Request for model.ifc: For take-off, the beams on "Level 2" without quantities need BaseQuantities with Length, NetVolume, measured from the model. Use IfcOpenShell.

First a look at what the model holds.

```python
import ifcopenshell
import ifcopenshell.util.element
import ifcopenshell.util.unit

model = ifcopenshell.open("model.ifc")
print(model.schema)
for unit_type in ("LENGTHUNIT", "AREAUNIT", "VOLUMEUNIT"):
    print(unit_type, ifcopenshell.util.unit.calculate_unit_scale(model, unit_type))
storey = next(s for s in model.by_type("IfcBuildingStorey") if s.Name == "Level 2")
beams = [e for e in ifcopenshell.util.element.get_decomposition(storey) if e.is_a("IfcBeam")]
for e in sorted(beams, key=lambda e: e.id()):
    print(e.id(), e.is_a(), e.Name, list(ifcopenshell.util.element.get_psets(e, qtos_only=True)), sep=" | ")
```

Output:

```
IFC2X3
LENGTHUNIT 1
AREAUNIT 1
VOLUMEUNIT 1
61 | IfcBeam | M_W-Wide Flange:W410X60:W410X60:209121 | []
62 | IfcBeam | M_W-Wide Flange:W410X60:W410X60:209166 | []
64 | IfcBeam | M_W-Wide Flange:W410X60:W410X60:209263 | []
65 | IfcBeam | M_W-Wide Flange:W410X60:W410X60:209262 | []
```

```python
import ifcopenshell
import ifcopenshell.api.pset
import ifcopenshell.geom
import ifcopenshell.util.element
import ifcopenshell.util.shape
import ifcopenshell.util.unit

model = ifcopenshell.open("model.ifc")
unit_scale = ifcopenshell.util.unit.calculate_unit_scale(model)
volume_scale = ifcopenshell.util.unit.calculate_unit_scale(model, "VOLUMEUNIT")
settings = ifcopenshell.geom.settings()

storey = next(s for s in model.by_type("IfcBuildingStorey") if s.Name == "Level 2")
beams = [e for e in ifcopenshell.util.element.get_decomposition(storey) if e.is_a("IfcBeam")]

for e in sorted(beams, key=lambda e: e.id()):
    if ifcopenshell.util.element.get_psets(e, qtos_only=True, should_inherit=False):
        continue
    # Geometry comes back in metres, in the element's own axes.
    shape = ifcopenshell.geom.create_shape(settings, e)
    values = {
        "Length": ifcopenshell.util.shape.get_max_xyz(shape.geometry) / unit_scale,
        "NetVolume": ifcopenshell.util.shape.get_volume(shape.geometry) / volume_scale,
    }
    qto = ifcopenshell.api.pset.add_qto(model, product=e, name="BaseQuantities")
    ifcopenshell.api.pset.edit_qto(model, qto=qto, properties=values)
    print(e.id(), {k: round(v, 3) for k, v in values.items()})

model.write("model-out.ifc")
```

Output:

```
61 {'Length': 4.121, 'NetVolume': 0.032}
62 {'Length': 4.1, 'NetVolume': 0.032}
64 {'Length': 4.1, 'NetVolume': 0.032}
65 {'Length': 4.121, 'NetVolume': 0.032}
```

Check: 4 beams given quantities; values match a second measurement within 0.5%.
